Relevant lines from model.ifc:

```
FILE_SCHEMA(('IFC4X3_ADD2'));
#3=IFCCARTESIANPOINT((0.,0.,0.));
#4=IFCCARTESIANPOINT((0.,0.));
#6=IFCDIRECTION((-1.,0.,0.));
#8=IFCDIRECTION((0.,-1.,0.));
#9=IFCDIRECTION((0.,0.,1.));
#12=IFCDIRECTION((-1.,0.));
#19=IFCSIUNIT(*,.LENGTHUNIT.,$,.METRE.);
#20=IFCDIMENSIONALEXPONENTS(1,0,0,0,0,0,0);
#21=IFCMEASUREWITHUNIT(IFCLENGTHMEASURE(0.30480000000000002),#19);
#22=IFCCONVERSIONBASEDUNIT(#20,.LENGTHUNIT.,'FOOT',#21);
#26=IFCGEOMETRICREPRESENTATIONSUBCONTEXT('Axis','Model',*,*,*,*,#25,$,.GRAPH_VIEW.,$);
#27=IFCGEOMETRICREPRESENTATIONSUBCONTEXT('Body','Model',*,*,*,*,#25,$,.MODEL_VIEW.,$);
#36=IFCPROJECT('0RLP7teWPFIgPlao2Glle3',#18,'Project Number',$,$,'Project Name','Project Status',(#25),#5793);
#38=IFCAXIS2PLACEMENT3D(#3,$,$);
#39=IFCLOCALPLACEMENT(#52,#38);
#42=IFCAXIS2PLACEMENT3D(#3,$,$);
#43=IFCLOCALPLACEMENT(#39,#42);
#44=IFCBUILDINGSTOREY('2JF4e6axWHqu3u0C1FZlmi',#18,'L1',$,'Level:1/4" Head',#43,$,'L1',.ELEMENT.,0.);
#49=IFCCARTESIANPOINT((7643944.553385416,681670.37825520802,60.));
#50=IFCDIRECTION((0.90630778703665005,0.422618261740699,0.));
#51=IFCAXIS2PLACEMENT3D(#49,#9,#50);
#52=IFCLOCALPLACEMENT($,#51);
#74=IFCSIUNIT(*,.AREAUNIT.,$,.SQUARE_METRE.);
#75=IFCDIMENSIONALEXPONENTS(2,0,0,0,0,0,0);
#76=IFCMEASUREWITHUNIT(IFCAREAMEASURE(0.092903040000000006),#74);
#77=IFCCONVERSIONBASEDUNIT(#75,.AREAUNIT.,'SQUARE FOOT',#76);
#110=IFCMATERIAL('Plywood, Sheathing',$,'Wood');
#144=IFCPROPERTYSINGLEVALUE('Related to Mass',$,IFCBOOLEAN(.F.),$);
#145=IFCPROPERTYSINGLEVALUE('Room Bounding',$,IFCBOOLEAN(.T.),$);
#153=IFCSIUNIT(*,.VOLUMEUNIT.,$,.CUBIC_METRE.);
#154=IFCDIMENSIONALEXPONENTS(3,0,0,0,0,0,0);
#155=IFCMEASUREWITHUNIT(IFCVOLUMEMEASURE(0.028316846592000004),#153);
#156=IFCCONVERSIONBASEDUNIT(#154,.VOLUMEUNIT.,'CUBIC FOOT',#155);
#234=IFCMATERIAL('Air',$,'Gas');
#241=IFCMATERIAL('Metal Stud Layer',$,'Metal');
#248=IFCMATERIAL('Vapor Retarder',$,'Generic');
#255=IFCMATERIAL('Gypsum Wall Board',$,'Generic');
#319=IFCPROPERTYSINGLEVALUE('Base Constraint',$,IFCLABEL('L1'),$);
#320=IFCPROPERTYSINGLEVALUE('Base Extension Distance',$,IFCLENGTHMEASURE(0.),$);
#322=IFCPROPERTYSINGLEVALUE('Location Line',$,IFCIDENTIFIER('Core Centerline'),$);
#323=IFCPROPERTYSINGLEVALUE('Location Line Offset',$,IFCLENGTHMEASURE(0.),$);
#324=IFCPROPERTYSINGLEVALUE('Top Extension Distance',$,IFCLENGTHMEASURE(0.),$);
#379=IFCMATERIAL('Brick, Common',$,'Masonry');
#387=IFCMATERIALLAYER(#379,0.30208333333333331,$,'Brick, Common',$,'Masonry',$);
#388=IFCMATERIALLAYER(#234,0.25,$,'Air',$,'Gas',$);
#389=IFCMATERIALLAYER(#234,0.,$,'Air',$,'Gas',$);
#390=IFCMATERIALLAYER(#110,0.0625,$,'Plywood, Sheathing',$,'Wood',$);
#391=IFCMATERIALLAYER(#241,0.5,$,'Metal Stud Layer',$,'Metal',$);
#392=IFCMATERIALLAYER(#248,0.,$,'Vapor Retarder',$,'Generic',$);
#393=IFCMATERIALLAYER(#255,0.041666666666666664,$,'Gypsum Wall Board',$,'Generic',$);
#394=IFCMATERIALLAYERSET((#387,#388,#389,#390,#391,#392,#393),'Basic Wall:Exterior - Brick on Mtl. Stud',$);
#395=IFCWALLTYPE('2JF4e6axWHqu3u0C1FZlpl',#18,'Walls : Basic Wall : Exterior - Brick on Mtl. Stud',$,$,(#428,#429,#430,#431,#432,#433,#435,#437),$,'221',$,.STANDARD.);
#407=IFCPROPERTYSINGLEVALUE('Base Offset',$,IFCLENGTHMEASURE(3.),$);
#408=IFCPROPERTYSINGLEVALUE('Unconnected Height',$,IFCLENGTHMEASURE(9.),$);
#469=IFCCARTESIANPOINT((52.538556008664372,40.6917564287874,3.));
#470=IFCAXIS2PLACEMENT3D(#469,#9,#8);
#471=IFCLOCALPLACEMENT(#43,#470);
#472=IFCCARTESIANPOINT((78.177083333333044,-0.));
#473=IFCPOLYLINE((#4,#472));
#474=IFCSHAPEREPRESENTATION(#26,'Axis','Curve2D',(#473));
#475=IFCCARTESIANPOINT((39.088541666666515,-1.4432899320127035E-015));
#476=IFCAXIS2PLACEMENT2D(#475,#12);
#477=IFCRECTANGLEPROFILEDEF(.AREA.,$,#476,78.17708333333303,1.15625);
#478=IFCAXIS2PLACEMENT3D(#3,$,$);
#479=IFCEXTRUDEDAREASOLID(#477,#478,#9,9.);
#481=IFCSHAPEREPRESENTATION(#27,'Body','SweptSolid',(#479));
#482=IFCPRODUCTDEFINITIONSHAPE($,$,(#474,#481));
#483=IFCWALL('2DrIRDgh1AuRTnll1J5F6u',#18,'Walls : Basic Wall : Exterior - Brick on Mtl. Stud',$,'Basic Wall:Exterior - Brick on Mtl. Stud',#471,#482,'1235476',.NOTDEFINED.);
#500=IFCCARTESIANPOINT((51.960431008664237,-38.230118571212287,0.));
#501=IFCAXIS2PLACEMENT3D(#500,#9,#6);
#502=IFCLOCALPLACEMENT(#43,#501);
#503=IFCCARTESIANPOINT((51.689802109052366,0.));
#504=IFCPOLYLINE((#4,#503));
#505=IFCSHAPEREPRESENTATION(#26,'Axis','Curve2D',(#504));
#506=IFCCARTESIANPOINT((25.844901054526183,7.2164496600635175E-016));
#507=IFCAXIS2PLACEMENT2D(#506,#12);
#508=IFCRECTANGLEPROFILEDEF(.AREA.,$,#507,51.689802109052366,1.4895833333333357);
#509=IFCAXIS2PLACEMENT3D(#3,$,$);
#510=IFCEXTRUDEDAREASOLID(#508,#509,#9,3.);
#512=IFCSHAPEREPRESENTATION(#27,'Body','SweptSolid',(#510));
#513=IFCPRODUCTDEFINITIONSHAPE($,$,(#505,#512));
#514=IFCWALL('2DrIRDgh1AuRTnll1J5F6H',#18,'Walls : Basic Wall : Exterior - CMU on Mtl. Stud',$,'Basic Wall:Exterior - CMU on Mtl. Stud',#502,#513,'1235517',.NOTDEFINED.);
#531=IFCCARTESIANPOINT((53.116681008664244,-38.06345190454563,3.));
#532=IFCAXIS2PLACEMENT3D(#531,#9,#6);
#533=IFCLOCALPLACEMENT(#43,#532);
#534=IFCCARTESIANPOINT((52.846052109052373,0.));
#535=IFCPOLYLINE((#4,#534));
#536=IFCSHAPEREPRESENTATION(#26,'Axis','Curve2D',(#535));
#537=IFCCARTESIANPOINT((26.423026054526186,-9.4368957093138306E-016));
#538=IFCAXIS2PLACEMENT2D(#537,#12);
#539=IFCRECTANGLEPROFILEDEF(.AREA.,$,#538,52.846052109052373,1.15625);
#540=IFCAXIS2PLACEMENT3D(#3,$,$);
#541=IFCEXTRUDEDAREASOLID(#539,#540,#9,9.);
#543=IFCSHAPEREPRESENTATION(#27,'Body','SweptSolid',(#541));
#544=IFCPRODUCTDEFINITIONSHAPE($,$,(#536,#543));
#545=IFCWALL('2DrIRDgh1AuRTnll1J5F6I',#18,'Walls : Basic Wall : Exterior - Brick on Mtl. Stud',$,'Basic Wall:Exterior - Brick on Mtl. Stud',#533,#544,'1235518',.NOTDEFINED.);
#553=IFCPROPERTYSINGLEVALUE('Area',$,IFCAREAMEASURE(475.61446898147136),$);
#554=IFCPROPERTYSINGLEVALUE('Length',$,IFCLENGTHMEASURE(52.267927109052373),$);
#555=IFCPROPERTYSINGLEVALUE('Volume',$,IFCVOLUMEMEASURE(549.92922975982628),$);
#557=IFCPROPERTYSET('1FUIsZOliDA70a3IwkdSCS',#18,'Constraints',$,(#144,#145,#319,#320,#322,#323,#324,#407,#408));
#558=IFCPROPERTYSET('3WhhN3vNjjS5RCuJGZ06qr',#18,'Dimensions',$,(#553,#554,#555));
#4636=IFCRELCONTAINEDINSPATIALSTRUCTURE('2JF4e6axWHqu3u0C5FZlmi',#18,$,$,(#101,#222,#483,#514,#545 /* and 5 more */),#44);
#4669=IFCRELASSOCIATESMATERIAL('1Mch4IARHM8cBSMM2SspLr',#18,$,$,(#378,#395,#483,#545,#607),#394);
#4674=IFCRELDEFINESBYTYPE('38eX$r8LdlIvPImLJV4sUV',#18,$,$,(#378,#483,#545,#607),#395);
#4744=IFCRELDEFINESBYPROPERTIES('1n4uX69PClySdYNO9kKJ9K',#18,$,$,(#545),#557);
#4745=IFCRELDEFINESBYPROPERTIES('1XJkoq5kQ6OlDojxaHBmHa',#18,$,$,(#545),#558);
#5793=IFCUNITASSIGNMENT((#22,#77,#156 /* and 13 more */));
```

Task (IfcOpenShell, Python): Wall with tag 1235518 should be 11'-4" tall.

```python
import ifcopenshell
import ifcopenshell.api.pset
import ifcopenshell.geom
import ifcopenshell.util.element
import ifcopenshell.util.representation
import ifcopenshell.util.shape
import ifcopenshell.util.unit

model = ifcopenshell.open("model.ifc")
unit_scale = ifcopenshell.util.unit.calculate_unit_scale(model)
area_scale = ifcopenshell.util.unit.calculate_unit_scale(model, "AREAUNIT")
volume_scale = ifcopenshell.util.unit.calculate_unit_scale(model, "VOLUMEUNIT")
settings = ifcopenshell.geom.settings()


def volume(element):
    """Net volume in cubic metres, openings subtracted."""
    shape = ifcopenshell.geom.create_shape(settings, element)
    return ifcopenshell.util.shape.get_volume(shape.geometry)


wall = model.by_guid("2DrIRDgh1AuRTnll1J5F6I")
before = volume(wall)

body = ifcopenshell.util.representation.get_representation(wall, "Model", "Body")
solid = body.Items[0]
old_height = solid.Depth
solid.Depth = 136 * 0.0254 / unit_scale
after = volume(wall)
thickness = 0.3524  # wall thickness in metres

# Update the stored height, areas and volumes.
pset = model.by_id(ifcopenshell.util.element.get_pset(wall, "Constraints", should_inherit=False)["id"])
ifcopenshell.api.pset.edit_pset(model, pset=pset, properties={
    "Unconnected Height": model.create_entity("IfcLengthMeasure", solid.Depth),
})
pset = model.by_id(ifcopenshell.util.element.get_pset(wall, "Dimensions", should_inherit=False)["id"])
ifcopenshell.api.pset.edit_pset(model, pset=pset, properties={
    "Area": model.create_entity("IfcAreaMeasure", after / thickness / area_scale),
    "Volume": model.create_entity("IfcVolumeMeasure", after / volume_scale),
})

print(f"height {old_height:g} -> {solid.Depth:g}, volume {before:.3f} -> {after:.3f} m3")

model.write("model_rev.ifc")
```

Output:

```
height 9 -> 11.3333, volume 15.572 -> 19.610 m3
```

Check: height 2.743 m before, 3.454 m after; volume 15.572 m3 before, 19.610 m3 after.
